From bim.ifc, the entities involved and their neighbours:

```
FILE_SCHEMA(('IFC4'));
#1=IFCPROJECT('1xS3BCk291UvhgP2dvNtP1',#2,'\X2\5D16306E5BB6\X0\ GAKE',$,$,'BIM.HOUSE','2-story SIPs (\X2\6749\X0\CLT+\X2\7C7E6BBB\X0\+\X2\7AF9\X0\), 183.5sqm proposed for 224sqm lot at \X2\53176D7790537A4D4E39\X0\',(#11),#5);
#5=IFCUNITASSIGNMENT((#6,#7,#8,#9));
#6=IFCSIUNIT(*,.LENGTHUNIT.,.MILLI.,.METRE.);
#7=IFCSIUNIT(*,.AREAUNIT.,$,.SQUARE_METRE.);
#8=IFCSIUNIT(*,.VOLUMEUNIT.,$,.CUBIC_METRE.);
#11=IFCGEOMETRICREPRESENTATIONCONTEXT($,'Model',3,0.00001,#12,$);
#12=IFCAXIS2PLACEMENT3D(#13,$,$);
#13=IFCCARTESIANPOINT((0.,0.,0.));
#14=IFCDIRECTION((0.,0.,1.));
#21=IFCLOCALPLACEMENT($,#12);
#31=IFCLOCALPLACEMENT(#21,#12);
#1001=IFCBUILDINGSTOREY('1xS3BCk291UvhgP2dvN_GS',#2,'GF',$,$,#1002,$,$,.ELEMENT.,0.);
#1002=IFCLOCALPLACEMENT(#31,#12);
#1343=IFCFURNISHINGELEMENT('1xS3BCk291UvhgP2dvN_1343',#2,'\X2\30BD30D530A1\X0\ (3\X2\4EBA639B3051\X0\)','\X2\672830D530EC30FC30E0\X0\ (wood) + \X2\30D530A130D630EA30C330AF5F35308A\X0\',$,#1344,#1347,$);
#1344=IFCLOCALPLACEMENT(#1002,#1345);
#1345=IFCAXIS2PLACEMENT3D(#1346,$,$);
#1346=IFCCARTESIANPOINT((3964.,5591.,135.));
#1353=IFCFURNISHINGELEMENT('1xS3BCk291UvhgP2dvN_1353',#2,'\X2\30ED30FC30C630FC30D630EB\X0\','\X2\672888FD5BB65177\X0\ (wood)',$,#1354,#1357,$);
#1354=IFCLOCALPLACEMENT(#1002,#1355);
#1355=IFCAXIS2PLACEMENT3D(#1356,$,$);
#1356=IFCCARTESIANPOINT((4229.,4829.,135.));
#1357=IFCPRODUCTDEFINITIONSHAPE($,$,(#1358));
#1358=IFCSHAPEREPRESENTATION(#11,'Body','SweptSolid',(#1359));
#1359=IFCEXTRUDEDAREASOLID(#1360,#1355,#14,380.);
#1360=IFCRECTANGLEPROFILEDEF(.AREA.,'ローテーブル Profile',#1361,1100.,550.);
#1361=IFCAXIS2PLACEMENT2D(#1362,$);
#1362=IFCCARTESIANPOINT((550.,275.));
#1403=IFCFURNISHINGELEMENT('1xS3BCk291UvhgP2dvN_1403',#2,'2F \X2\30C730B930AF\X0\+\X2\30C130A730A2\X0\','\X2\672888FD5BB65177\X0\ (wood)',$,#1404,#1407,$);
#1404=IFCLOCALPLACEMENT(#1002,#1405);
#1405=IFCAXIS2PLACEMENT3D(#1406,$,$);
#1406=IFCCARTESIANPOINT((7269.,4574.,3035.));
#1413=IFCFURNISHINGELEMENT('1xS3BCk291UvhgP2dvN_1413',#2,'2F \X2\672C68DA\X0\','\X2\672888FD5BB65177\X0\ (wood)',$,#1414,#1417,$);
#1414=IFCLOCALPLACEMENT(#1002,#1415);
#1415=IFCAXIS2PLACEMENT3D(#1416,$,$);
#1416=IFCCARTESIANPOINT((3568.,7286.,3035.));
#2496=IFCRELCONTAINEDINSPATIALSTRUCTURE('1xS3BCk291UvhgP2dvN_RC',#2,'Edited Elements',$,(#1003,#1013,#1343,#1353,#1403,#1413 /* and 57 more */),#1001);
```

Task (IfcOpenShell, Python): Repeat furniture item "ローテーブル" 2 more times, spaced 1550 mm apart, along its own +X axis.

```python
import ifcopenshell
import ifcopenshell.api.geometry
import ifcopenshell.api.root
import ifcopenshell.util.element
import ifcopenshell.util.placement
import ifcopenshell.util.unit

model = ifcopenshell.open("bim.ifc")
unit_scale = ifcopenshell.util.unit.calculate_unit_scale(model)


def reuse_history(source, copy):
    """copy_class also copies each property set's owner history, people and application; keep the originals."""
    for rel in copy.IsDefinedBy:
        if rel.is_a("IfcRelDefinesByProperties") and (history := rel.RelatingPropertyDefinition.OwnerHistory):
            rel.RelatingPropertyDefinition.OwnerHistory = source.OwnerHistory
            ifcopenshell.util.element.remove_deep2(model, history)


source = model.by_guid("1xS3BCk291UvhgP2dvN_1353")
base = ifcopenshell.util.placement.get_local_placement(source.ObjectPlacement)
step = base[:3, 0] * 1.55 / unit_scale

for i in range(1, 3):
    copy = ifcopenshell.api.root.copy_class(model, product=source)
    copy.Representation = ifcopenshell.util.element.copy_deep(
        model, source.Representation, exclude=["IfcGeometricRepresentationContext", "IfcRepresentationMap"]
    )
    reuse_history(source, copy)
    matrix = base.copy()
    matrix[:3, 3] += i * step
    print("added at", matrix[:3, 3].round(3) + 0.0)
    ifcopenshell.api.geometry.edit_object_placement(model, product=copy, matrix=matrix, is_si=False)

model.write("bim_edited.ifc")
```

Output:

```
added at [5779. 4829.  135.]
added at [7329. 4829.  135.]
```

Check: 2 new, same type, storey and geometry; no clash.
